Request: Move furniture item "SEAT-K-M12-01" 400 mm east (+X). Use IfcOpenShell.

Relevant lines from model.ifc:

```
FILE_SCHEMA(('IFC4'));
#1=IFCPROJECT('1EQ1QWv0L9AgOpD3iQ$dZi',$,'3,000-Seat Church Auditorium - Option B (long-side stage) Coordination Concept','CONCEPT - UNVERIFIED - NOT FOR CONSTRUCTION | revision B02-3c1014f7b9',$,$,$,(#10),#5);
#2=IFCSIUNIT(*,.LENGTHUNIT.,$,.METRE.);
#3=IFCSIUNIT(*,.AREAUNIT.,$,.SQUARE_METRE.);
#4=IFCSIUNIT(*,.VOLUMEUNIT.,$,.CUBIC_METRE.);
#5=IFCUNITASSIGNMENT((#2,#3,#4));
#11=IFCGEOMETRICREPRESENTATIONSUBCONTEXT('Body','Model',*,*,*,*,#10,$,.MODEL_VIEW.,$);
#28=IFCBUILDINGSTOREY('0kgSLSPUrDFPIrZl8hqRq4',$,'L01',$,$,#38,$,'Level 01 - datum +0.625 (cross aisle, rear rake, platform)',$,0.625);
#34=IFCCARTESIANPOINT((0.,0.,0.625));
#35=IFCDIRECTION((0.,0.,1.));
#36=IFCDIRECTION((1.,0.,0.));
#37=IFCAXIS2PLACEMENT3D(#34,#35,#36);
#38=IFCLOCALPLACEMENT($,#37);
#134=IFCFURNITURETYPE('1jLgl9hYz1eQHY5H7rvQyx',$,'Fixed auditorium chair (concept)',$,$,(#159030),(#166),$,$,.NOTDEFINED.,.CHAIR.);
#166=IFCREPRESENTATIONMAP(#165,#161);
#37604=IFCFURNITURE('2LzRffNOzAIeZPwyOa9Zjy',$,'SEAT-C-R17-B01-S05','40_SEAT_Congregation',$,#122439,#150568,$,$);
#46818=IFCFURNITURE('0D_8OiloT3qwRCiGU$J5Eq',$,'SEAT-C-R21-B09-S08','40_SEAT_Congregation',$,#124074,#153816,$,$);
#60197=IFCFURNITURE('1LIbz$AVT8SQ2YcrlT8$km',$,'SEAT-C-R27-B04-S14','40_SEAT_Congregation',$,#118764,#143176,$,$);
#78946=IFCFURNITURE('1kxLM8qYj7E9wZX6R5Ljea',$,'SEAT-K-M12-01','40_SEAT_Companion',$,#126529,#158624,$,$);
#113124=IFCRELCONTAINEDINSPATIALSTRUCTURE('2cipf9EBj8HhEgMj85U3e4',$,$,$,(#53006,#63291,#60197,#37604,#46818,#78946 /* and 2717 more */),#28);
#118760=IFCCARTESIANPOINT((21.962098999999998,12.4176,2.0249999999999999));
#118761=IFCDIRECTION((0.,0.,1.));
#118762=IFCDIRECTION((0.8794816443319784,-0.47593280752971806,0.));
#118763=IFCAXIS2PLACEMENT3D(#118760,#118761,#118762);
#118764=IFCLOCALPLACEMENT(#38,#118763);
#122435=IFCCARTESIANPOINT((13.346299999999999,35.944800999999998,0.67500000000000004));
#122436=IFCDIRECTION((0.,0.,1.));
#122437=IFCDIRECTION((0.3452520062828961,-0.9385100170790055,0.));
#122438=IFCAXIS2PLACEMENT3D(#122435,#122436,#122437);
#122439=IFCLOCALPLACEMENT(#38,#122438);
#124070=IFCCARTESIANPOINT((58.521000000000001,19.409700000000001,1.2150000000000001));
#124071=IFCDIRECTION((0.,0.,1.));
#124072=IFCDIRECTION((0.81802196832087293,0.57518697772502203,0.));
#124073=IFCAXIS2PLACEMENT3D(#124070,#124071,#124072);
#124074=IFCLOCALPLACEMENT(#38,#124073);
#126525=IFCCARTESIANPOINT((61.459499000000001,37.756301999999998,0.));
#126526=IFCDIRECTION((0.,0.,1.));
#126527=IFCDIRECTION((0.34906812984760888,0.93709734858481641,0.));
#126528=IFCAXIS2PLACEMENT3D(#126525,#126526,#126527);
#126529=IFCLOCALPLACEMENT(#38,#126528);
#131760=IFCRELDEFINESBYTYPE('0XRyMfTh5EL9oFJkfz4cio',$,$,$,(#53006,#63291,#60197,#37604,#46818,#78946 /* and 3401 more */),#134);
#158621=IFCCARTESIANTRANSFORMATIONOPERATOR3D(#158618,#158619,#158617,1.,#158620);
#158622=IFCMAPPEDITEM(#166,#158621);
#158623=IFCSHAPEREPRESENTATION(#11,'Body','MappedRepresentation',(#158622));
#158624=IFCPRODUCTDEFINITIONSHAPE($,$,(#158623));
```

```python
import ifcopenshell
import ifcopenshell.api.geometry
import ifcopenshell.util.placement
import ifcopenshell.util.unit

model = ifcopenshell.open("model.ifc")
unit_scale = ifcopenshell.util.unit.calculate_unit_scale(model)

item = model.by_guid("1kxLM8qYj7E9wZX6R5Ljea")
matrix = ifcopenshell.util.placement.get_local_placement(item.ObjectPlacement)
matrix[0, 3] += 0.4 / unit_scale
ifcopenshell.api.geometry.edit_object_placement(model, product=item, matrix=matrix, is_si=False)

print(ifcopenshell.util.placement.get_local_placement(item.ObjectPlacement).round(3) + 0.0)

model.write("model_edited.ifc")
```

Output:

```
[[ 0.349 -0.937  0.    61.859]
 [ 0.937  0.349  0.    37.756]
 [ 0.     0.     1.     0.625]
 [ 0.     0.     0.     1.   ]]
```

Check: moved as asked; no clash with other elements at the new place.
